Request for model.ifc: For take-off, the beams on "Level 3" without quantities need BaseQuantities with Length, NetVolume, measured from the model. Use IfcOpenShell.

First a look at what the model holds.

```python
import ifcopenshell
import ifcopenshell.util.element
import ifcopenshell.util.unit

model = ifcopenshell.open("model.ifc")
print(model.schema)
for unit_type in ("LENGTHUNIT", "AREAUNIT", "VOLUMEUNIT"):
    print(unit_type, ifcopenshell.util.unit.calculate_unit_scale(model, unit_type))
storey = next(s for s in model.by_type("IfcBuildingStorey") if s.Name == "Level 3")
beams = [e for e in ifcopenshell.util.element.get_decomposition(storey) if e.is_a("IfcBeam")]
for e in sorted(beams, key=lambda e: e.id()):
    print(e.id(), e.is_a(), e.Name, list(ifcopenshell.util.element.get_psets(e, qtos_only=True)), sep=" | ")
```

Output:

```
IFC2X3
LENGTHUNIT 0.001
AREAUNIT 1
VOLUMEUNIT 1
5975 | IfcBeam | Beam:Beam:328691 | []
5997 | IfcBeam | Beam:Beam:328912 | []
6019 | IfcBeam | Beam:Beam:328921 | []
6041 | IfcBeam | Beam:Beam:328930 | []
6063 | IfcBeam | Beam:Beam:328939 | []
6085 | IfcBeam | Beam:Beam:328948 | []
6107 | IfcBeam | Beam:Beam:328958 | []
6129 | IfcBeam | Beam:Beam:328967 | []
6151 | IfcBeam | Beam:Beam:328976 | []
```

```python
import ifcopenshell
import ifcopenshell.api.pset
import ifcopenshell.geom
import ifcopenshell.util.element
import ifcopenshell.util.shape
import ifcopenshell.util.unit

model = ifcopenshell.open("model.ifc")
unit_scale = ifcopenshell.util.unit.calculate_unit_scale(model)
volume_scale = ifcopenshell.util.unit.calculate_unit_scale(model, "VOLUMEUNIT")
settings = ifcopenshell.geom.settings()

storey = next(s for s in model.by_type("IfcBuildingStorey") if s.Name == "Level 3")
beams = [e for e in ifcopenshell.util.element.get_decomposition(storey) if e.is_a("IfcBeam")]

for e in sorted(beams, key=lambda e: e.id()):
    if ifcopenshell.util.element.get_psets(e, qtos_only=True, should_inherit=False):
        continue
    # Geometry comes back in metres, in the element's own axes.
    shape = ifcopenshell.geom.create_shape(settings, e)
    values = {
        "Length": ifcopenshell.util.shape.get_max_xyz(shape.geometry) / unit_scale,
        "NetVolume": ifcopenshell.util.shape.get_volume(shape.geometry) / volume_scale,
    }
    qto = ifcopenshell.api.pset.add_qto(model, product=e, name="BaseQuantities")
    ifcopenshell.api.pset.edit_qto(model, qto=qto, properties=values)
    print(e.id(), {k: round(v, 3) for k, v in values.items()})

model.write("model_v2.ifc")
```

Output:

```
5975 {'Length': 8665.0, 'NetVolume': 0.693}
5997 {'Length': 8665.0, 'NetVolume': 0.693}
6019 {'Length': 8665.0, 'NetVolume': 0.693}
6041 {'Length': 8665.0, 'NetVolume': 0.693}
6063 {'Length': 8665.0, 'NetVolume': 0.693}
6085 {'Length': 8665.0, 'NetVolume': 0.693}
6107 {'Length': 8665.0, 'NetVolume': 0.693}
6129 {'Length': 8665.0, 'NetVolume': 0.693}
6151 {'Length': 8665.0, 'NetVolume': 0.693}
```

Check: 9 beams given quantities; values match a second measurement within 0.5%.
